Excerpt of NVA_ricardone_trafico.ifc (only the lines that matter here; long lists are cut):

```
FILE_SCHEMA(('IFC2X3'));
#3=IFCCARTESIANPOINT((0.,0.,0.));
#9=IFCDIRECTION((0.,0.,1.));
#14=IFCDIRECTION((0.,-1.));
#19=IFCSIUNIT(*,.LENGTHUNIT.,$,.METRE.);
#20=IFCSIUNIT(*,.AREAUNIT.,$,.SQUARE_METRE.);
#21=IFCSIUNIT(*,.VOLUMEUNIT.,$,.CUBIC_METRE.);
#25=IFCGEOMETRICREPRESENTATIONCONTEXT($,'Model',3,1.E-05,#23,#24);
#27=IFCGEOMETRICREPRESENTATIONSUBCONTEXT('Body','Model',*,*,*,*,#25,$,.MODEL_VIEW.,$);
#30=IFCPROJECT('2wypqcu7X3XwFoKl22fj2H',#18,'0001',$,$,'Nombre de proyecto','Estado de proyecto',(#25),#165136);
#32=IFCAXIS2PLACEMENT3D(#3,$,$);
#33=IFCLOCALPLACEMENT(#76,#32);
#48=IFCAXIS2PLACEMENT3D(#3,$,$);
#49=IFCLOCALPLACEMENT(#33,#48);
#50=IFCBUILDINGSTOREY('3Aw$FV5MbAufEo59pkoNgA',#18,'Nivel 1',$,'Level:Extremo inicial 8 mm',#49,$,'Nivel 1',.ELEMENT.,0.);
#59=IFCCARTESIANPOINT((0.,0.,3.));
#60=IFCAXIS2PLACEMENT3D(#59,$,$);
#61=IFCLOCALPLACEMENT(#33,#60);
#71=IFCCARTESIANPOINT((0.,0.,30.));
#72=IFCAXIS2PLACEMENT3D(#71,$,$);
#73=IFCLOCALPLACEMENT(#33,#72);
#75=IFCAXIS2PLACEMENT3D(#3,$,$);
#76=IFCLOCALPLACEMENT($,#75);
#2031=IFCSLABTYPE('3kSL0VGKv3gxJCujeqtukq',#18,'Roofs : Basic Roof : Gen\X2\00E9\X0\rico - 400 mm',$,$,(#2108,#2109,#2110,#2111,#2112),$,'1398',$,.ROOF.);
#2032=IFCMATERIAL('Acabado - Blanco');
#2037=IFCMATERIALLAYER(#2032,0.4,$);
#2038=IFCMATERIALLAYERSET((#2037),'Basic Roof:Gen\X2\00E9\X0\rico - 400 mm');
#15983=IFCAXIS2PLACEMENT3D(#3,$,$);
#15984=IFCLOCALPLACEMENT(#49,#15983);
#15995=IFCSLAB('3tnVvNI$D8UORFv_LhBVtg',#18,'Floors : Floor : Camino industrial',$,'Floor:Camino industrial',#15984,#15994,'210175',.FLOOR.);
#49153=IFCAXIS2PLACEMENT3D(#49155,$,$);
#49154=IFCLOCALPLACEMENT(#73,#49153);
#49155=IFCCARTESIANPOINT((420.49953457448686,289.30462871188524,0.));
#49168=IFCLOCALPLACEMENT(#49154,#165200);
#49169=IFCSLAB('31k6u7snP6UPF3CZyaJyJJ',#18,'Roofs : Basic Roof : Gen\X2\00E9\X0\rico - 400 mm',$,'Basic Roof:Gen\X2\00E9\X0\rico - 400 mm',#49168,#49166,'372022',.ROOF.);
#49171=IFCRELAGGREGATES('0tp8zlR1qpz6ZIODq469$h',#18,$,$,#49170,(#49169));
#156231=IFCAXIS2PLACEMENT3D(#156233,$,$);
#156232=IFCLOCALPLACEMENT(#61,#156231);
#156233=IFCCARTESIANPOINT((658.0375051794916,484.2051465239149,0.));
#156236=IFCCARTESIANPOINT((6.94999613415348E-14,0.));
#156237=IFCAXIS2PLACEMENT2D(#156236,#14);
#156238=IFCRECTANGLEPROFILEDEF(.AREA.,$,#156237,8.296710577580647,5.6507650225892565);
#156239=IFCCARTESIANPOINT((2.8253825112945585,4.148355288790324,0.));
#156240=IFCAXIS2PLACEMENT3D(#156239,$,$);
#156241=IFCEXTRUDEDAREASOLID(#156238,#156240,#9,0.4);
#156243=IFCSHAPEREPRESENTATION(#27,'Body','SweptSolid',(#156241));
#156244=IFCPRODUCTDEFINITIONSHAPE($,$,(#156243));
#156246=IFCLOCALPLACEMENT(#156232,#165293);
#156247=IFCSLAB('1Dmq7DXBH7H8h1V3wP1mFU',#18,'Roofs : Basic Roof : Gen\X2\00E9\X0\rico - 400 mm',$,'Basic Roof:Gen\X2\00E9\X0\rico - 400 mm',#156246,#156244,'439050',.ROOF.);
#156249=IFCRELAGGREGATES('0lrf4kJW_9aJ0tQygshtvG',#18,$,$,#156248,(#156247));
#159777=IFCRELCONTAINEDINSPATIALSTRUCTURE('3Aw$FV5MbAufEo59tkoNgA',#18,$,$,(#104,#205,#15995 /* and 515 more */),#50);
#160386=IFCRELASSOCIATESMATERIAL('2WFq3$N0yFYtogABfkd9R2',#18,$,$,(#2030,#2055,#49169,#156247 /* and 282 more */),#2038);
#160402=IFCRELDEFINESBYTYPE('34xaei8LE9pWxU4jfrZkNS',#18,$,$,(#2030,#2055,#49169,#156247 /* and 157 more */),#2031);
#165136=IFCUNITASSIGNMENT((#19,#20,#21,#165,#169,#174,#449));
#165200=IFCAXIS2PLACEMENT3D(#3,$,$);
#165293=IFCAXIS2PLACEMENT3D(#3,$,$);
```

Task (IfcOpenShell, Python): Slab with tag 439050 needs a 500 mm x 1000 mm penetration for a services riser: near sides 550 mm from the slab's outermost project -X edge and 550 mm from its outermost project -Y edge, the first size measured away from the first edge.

```python
import numpy as np
import ifcopenshell
import ifcopenshell.api.feature
import ifcopenshell.api.geometry
import ifcopenshell.api.root
import ifcopenshell.geom
import ifcopenshell.util.placement
import ifcopenshell.util.representation
import ifcopenshell.util.shape
import ifcopenshell.util.unit

model = ifcopenshell.open("NVA_ricardone_trafico.ifc")
unit_scale = ifcopenshell.util.unit.calculate_unit_scale(model)
settings = ifcopenshell.geom.settings()


def volume(element):
    """Net volume in cubic metres, openings subtracted."""
    shape = ifcopenshell.geom.create_shape(settings, element)
    return ifcopenshell.util.shape.get_volume(shape.geometry)


slab = model.by_guid("1Dmq7DXBH7H8h1V3wP1mFU")
before = volume(slab)

# Extent in the slab's own axes, in metres. The edges named are its -X and -Y sides.
slab_shape = ifcopenshell.geom.create_shape(settings, slab)
vertices = ifcopenshell.util.shape.get_vertices(slab_shape.geometry)
x_min, y_min, bottom = vertices.min(axis=0)
top = vertices[:, 2].max()

opening = ifcopenshell.api.root.create_entity(model, ifc_class="IfcOpeningElement", name="Services riser opening")
context = ifcopenshell.util.representation.get_context(model, "Model", "Body", "MODEL_VIEW")
width, depth = 0.5, 1
outline = [(0.0, 0.0), (width, 0.0), (width, depth), (0.0, depth), (0.0, 0.0)]
# Overshoot both faces by 50 mm so the cut is clean.
shape = ifcopenshell.api.geometry.add_slab_representation(
    model, context=context, depth=top - bottom + 0.1, polyline=outline
)
ifcopenshell.api.geometry.assign_representation(model, product=opening, representation=shape)

matrix = ifcopenshell.util.placement.get_local_placement(slab.ObjectPlacement)
matrix[:, 3] = matrix @ np.append(np.array([x_min + 0.55, y_min + 0.55, bottom - 0.05]) / unit_scale, 1.0)
ifcopenshell.api.geometry.edit_object_placement(model, product=opening, matrix=matrix, is_si=False)
ifcopenshell.api.feature.add_feature(model, feature=opening, element=slab)

after = volume(slab)

print(f"slab volume {before:.3f} -> {after:.3f} m3")

model.write("NVA_ricardone_trafico_v2.ifc")
```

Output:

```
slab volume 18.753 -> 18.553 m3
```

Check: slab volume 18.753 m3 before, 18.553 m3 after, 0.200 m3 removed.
